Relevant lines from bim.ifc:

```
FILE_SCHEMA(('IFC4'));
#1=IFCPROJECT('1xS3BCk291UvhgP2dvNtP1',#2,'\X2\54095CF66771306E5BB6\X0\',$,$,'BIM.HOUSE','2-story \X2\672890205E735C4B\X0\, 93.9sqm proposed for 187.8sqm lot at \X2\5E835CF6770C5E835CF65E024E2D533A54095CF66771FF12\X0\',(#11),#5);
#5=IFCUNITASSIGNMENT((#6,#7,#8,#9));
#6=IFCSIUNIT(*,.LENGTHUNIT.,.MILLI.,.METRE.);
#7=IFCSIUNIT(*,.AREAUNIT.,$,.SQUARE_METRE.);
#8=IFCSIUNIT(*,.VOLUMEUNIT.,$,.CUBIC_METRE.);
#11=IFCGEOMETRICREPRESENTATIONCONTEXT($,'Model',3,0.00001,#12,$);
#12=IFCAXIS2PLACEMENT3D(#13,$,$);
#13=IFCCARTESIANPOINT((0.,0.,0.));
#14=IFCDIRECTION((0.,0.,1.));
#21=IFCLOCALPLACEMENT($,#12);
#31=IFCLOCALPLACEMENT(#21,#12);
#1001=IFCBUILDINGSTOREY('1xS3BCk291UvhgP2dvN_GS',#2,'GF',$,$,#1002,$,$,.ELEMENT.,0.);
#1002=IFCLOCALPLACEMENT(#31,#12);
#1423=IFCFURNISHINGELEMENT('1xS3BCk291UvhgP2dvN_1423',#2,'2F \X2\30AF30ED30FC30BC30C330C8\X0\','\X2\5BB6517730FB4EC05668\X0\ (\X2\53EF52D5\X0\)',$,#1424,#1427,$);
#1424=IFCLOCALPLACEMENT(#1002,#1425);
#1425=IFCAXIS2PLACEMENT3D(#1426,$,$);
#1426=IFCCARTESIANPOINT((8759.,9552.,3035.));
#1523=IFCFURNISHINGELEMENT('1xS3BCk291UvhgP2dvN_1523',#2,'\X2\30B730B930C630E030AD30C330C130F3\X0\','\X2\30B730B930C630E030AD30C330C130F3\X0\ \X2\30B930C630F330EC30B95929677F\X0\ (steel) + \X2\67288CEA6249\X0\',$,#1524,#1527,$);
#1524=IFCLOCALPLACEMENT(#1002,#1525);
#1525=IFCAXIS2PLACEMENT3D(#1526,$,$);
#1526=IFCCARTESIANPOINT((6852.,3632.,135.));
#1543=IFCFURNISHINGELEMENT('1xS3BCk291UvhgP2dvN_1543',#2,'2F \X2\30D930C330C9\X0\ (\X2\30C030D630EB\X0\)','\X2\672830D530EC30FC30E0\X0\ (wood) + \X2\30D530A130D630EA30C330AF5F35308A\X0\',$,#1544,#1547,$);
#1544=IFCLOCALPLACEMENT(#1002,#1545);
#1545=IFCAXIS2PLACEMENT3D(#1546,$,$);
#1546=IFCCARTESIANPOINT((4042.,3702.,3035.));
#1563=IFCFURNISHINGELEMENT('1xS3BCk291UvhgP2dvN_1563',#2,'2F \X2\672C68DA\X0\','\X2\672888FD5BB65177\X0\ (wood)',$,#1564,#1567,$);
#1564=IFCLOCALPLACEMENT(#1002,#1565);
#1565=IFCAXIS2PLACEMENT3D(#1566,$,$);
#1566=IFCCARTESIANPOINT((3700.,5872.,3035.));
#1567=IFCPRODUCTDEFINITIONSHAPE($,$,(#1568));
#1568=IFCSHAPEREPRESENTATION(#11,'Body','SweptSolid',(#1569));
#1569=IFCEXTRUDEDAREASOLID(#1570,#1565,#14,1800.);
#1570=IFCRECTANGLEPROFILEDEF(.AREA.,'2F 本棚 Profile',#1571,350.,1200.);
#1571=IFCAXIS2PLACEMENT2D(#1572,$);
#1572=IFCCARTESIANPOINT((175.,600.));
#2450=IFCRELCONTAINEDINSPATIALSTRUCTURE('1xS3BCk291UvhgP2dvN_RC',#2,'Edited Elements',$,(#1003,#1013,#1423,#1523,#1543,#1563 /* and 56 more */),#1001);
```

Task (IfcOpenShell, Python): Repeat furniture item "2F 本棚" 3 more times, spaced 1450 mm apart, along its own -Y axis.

```python
import ifcopenshell
import ifcopenshell.api.geometry
import ifcopenshell.api.root
import ifcopenshell.util.element
import ifcopenshell.util.placement
import ifcopenshell.util.unit

model = ifcopenshell.open("bim.ifc")
unit_scale = ifcopenshell.util.unit.calculate_unit_scale(model)


def reuse_history(source, copy):
    """copy_class also copies each property set's owner history, people and application; keep the originals."""
    for rel in copy.IsDefinedBy:
        if rel.is_a("IfcRelDefinesByProperties") and (history := rel.RelatingPropertyDefinition.OwnerHistory):
            rel.RelatingPropertyDefinition.OwnerHistory = source.OwnerHistory
            ifcopenshell.util.element.remove_deep2(model, history)


source = model.by_id(1563)
base = ifcopenshell.util.placement.get_local_placement(source.ObjectPlacement)
step = -base[:3, 1] * 1.45 / unit_scale

for i in range(1, 4):
    copy = ifcopenshell.api.root.copy_class(model, product=source)
    copy.Representation = ifcopenshell.util.element.copy_deep(
        model, source.Representation, exclude=["IfcGeometricRepresentationContext", "IfcRepresentationMap"]
    )
    reuse_history(source, copy)
    matrix = base.copy()
    matrix[:3, 3] += i * step
    print("added at", matrix[:3, 3].round(3) + 0.0)
    ifcopenshell.api.geometry.edit_object_placement(model, product=copy, matrix=matrix, is_si=False)

model.write("bim_rev.ifc")
```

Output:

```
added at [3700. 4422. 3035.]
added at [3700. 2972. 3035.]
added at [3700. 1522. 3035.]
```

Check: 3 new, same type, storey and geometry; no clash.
